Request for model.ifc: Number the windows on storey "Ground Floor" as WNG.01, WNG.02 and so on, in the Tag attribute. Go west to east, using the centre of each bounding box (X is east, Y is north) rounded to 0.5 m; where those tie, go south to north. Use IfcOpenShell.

First a look at what the model holds.

```python
import ifcopenshell
import ifcopenshell.util.element
import ifcopenshell.util.placement

model = ifcopenshell.open("model.ifc")
print(model.schema)
storey = next(s for s in model.by_type("IfcBuildingStorey") if s.Name == "Ground Floor")
windows = [e for e in ifcopenshell.util.element.get_decomposition(storey) if e.is_a("IfcWindow")]
for e in sorted(windows, key=lambda e: e.id()):
    origin = ifcopenshell.util.placement.get_local_placement(e.ObjectPlacement)[:3, 3]
    print(e.id(), e.Tag, e.Name, origin.round(2) + 0.0, sep=" | ")
```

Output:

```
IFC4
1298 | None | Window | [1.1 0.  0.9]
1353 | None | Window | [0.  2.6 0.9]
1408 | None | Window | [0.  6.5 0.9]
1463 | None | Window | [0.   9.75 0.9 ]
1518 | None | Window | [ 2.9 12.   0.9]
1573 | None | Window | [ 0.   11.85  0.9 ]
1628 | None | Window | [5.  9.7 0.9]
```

```python
import ifcopenshell
import ifcopenshell.geom
import ifcopenshell.util.element
import ifcopenshell.util.shape

model = ifcopenshell.open("model.ifc")
settings = ifcopenshell.geom.settings()
settings.set("use-world-coords", True)


def centre(element):
    shape = ifcopenshell.geom.create_shape(settings, element)
    return ifcopenshell.util.shape.get_bbox_centroid(shape.geometry)


storey = next(s for s in model.by_type("IfcBuildingStorey") if s.Name == "Ground Floor")
windows = [e for e in ifcopenshell.util.element.get_decomposition(storey) if e.is_a("IfcWindow")]

# Insertion points can sit at a corner or the storey origin, so sort by the geometry (in metres).
centres = {e: centre(e) for e in windows}
windows.sort(key=lambda e: (round(centres[e][0] / 0.5), centres[e][1]))

for i, e in enumerate(windows, start=1):
    number = f"WNG.{i:02d}"
    e.Tag = number
    print(e.id(), number)

model.write("model_v2.ifc")
```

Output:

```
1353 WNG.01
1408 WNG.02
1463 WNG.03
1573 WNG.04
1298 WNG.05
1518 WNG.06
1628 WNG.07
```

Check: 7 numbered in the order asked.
